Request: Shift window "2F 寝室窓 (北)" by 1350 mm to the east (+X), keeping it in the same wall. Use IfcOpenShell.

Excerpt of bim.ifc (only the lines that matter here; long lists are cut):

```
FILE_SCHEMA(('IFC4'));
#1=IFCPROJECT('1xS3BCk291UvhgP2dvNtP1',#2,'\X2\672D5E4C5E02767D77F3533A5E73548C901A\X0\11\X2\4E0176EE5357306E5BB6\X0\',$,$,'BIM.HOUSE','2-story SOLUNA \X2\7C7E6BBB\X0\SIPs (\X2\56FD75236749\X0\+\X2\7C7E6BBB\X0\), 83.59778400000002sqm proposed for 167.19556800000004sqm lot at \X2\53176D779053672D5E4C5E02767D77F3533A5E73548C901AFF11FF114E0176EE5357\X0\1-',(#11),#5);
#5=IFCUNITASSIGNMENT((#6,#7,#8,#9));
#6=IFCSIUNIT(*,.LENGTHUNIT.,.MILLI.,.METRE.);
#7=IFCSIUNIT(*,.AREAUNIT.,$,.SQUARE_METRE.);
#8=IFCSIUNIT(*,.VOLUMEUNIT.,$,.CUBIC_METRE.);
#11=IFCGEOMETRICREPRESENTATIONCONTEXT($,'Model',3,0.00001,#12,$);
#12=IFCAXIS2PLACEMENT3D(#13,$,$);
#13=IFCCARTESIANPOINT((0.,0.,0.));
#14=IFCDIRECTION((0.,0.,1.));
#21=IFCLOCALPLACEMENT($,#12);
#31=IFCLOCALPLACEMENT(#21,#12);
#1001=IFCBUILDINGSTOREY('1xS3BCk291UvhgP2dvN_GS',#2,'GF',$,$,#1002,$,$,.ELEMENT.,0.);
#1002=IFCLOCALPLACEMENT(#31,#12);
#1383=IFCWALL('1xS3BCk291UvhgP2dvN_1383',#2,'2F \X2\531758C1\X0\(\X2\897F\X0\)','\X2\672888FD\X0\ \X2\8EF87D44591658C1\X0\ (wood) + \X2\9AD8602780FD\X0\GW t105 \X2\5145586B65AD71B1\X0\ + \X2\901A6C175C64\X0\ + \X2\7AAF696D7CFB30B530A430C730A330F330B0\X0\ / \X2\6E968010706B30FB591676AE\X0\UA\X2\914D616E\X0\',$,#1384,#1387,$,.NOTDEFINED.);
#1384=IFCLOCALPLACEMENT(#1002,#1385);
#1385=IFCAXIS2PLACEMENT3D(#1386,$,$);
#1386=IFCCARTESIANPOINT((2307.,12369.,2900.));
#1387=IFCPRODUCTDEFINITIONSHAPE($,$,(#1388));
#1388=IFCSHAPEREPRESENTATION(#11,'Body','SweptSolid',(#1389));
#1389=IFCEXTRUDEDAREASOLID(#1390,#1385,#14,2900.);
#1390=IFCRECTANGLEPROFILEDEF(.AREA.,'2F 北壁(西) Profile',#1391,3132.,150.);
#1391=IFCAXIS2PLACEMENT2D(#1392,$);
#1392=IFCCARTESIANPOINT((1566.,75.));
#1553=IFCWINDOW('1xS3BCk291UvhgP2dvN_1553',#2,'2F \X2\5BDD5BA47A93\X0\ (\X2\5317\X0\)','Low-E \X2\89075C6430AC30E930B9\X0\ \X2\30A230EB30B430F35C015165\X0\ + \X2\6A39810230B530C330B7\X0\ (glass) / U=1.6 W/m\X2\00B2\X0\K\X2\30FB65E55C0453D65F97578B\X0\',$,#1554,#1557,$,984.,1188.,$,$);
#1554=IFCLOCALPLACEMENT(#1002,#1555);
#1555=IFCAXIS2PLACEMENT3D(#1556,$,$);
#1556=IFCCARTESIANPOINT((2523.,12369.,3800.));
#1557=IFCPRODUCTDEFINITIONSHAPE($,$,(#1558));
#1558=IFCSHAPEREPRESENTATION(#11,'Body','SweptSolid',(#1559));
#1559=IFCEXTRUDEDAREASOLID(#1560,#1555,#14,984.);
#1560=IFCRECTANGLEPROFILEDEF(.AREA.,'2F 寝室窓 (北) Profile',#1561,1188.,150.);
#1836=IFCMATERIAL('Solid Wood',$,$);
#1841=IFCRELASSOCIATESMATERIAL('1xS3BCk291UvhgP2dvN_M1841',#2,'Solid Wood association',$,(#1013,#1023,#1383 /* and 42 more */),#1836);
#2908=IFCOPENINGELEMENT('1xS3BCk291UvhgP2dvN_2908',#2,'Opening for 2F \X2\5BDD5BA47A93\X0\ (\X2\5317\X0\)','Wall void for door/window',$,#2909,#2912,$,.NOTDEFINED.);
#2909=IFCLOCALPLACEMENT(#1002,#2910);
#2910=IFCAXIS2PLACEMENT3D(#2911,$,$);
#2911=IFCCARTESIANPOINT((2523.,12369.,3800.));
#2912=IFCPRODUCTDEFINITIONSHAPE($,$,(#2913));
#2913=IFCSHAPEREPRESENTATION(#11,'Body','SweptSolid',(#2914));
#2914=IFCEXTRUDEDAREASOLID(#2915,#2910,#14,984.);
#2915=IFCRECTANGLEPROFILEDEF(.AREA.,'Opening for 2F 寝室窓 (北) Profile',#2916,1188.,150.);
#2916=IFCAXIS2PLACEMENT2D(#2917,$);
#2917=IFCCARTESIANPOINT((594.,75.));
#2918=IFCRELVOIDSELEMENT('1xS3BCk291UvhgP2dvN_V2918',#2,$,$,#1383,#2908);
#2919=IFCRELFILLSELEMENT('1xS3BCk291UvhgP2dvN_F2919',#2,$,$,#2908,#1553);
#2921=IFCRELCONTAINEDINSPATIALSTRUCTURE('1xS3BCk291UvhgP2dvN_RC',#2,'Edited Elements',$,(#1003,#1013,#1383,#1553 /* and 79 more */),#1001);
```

```python
import ifcopenshell
import ifcopenshell.api.geometry
import ifcopenshell.util.placement

model = ifcopenshell.open("bim.ifc")

window = model.by_guid("1xS3BCk291UvhgP2dvN_1553")
opening = window.FillsVoids[0].RelatingOpeningElement
wall = opening.VoidsElements[0].RelatingBuildingElement

wall_matrix = ifcopenshell.util.placement.get_local_placement(wall.ObjectPlacement)
shift = wall_matrix[:3, 0] * 1350.0
before = ifcopenshell.util.placement.get_local_placement(window.ObjectPlacement)[:3, 3].copy()

# The window is not placed relative to its opening, so move both.
for product in (opening, window):
    matrix = ifcopenshell.util.placement.get_local_placement(product.ObjectPlacement)
    matrix[:3, 3] += shift
    ifcopenshell.api.geometry.edit_object_placement(model, product=product, matrix=matrix, is_si=False)

after = ifcopenshell.util.placement.get_local_placement(window.ObjectPlacement)[:3, 3]
print("window moved by", (after - before).round(3) + 0.0)

model.write("bim_updated.ifc")
```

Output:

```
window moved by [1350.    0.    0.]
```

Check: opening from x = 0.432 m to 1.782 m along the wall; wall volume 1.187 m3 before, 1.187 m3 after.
